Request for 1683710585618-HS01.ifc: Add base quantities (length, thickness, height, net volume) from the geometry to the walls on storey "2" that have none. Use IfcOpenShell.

First a look at what the model holds.

```python
import ifcopenshell
import ifcopenshell.util.element
import ifcopenshell.util.unit

model = ifcopenshell.open("1683710585618-HS01.ifc")
print(model.schema)
for unit_type in ("LENGTHUNIT", "AREAUNIT", "VOLUMEUNIT"):
    print(unit_type, ifcopenshell.util.unit.calculate_unit_scale(model, unit_type))
storey = next(s for s in model.by_type("IfcBuildingStorey") if s.Name == "2")
walls = [e for e in ifcopenshell.util.element.get_decomposition(storey) if e.is_a("IfcWall")]
for e in sorted(walls, key=lambda e: e.id()):
    print(e.id(), e.is_a(), e.Name, list(ifcopenshell.util.element.get_psets(e, qtos_only=True)), sep=" | ")
```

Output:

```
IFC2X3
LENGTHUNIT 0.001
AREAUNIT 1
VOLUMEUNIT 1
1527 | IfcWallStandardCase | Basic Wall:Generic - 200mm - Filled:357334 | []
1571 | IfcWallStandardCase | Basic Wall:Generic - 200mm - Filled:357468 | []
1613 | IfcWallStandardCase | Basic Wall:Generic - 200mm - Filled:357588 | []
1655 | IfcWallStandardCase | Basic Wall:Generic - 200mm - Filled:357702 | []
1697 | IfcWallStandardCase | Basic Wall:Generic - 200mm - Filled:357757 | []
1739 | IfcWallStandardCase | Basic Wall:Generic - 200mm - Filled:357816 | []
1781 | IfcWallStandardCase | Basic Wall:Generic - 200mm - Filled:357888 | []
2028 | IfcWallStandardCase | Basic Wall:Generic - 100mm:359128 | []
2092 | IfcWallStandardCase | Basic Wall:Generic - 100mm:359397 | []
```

```python
import ifcopenshell
import ifcopenshell.api.pset
import ifcopenshell.geom
import ifcopenshell.util.element
import ifcopenshell.util.shape
import ifcopenshell.util.unit

model = ifcopenshell.open("1683710585618-HS01.ifc")
unit_scale = ifcopenshell.util.unit.calculate_unit_scale(model)
volume_scale = ifcopenshell.util.unit.calculate_unit_scale(model, "VOLUMEUNIT")
settings = ifcopenshell.geom.settings()

storey = next(s for s in model.by_type("IfcBuildingStorey") if s.Name == "2")
walls = [e for e in ifcopenshell.util.element.get_decomposition(storey) if e.is_a("IfcWall")]

for e in sorted(walls, key=lambda e: e.id()):
    if ifcopenshell.util.element.get_psets(e, qtos_only=True, should_inherit=False):
        continue
    # Geometry comes back in metres, in the element's own axes.
    shape = ifcopenshell.geom.create_shape(settings, e)
    values = {
        "Length": ifcopenshell.util.shape.get_x(shape.geometry) / unit_scale,
        "Width": ifcopenshell.util.shape.get_y(shape.geometry) / unit_scale,
        "Height": ifcopenshell.util.shape.get_z(shape.geometry) / unit_scale,
        "NetVolume": ifcopenshell.util.shape.get_volume(shape.geometry) / volume_scale,
    }
    qto = ifcopenshell.api.pset.add_qto(model, product=e, name="BaseQuantities")
    ifcopenshell.api.pset.edit_qto(model, qto=qto, properties=values)
    print(e.id(), {k: round(v, 3) for k, v in values.items()})

model.write("1683710585618-HS01_rev.ifc")
```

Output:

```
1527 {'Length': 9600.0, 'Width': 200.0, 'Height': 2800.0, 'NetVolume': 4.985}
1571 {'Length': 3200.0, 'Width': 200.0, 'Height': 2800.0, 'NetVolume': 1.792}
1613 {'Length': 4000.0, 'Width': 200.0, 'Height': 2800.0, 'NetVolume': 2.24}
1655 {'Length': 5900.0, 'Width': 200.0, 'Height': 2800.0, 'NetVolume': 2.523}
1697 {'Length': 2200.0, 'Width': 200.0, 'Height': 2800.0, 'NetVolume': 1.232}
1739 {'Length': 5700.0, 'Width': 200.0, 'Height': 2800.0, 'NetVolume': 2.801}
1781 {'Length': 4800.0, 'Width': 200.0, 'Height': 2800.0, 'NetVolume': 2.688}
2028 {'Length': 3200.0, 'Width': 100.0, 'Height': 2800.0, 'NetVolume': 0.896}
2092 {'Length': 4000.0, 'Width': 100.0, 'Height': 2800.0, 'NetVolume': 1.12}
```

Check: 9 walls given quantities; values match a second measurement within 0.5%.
